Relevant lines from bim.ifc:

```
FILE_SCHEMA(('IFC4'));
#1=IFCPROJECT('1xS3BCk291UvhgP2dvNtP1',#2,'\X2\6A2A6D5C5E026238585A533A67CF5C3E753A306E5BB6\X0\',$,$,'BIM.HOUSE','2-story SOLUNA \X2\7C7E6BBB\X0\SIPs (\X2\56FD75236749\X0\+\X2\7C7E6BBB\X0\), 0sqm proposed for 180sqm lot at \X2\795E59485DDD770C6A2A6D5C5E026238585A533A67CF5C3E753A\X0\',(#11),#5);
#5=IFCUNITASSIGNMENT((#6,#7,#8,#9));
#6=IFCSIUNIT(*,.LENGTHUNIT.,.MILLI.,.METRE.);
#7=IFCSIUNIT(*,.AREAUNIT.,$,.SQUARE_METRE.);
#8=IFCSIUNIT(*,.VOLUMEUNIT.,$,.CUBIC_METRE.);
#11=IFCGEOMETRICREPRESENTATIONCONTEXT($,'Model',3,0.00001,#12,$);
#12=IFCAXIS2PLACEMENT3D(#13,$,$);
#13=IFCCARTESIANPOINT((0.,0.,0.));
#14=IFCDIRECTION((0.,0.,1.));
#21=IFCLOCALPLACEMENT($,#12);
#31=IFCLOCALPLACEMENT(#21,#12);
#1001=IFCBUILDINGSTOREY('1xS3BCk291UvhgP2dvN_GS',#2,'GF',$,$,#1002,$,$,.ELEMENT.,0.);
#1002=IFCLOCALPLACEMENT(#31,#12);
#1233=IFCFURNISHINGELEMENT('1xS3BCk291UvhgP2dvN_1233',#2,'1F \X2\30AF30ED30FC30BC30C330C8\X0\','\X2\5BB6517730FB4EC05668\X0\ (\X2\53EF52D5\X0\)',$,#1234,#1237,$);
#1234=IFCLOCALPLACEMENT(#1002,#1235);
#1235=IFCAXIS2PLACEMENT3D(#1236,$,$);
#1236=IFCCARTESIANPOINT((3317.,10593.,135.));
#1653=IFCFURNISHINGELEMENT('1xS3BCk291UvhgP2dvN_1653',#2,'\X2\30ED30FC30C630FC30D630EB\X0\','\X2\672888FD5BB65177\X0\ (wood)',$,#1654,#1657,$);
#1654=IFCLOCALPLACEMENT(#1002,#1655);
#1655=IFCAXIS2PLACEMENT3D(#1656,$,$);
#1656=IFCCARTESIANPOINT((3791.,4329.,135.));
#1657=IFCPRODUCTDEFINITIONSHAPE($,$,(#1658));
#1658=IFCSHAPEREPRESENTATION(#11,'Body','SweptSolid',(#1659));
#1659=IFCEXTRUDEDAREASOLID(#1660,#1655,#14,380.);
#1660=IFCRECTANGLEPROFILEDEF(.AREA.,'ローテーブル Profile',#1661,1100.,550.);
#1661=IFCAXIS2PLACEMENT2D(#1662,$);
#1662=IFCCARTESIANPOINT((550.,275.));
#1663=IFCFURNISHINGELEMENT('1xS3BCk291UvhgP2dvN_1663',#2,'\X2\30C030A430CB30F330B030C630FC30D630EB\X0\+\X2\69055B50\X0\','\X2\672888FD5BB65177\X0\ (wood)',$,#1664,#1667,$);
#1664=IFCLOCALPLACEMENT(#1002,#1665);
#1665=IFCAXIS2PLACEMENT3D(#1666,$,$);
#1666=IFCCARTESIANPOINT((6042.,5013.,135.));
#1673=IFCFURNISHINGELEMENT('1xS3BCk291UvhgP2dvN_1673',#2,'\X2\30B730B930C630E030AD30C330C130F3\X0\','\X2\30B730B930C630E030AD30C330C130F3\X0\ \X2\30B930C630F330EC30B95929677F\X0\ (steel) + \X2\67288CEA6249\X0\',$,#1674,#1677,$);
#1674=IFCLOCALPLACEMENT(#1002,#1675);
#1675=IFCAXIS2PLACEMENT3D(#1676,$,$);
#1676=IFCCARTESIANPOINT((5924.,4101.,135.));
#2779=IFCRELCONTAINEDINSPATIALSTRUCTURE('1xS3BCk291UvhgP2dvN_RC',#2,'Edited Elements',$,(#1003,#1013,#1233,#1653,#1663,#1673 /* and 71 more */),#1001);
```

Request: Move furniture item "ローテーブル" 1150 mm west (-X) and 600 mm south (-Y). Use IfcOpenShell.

```python
import ifcopenshell
import ifcopenshell.api.geometry
import ifcopenshell.util.placement

model = ifcopenshell.open("bim.ifc")

item = model.by_id(1653)
matrix = ifcopenshell.util.placement.get_local_placement(item.ObjectPlacement)
matrix[0, 3] -= 1150.0
matrix[1, 3] -= 600.0
ifcopenshell.api.geometry.edit_object_placement(model, product=item, matrix=matrix, is_si=False)

print(ifcopenshell.util.placement.get_local_placement(item.ObjectPlacement).round(3) + 0.0)

model.write("bim_rev.ifc")
```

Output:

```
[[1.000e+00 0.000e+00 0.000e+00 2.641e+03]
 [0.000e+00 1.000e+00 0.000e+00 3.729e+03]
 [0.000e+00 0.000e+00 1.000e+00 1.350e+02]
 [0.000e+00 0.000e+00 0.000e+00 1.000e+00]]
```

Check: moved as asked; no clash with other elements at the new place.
